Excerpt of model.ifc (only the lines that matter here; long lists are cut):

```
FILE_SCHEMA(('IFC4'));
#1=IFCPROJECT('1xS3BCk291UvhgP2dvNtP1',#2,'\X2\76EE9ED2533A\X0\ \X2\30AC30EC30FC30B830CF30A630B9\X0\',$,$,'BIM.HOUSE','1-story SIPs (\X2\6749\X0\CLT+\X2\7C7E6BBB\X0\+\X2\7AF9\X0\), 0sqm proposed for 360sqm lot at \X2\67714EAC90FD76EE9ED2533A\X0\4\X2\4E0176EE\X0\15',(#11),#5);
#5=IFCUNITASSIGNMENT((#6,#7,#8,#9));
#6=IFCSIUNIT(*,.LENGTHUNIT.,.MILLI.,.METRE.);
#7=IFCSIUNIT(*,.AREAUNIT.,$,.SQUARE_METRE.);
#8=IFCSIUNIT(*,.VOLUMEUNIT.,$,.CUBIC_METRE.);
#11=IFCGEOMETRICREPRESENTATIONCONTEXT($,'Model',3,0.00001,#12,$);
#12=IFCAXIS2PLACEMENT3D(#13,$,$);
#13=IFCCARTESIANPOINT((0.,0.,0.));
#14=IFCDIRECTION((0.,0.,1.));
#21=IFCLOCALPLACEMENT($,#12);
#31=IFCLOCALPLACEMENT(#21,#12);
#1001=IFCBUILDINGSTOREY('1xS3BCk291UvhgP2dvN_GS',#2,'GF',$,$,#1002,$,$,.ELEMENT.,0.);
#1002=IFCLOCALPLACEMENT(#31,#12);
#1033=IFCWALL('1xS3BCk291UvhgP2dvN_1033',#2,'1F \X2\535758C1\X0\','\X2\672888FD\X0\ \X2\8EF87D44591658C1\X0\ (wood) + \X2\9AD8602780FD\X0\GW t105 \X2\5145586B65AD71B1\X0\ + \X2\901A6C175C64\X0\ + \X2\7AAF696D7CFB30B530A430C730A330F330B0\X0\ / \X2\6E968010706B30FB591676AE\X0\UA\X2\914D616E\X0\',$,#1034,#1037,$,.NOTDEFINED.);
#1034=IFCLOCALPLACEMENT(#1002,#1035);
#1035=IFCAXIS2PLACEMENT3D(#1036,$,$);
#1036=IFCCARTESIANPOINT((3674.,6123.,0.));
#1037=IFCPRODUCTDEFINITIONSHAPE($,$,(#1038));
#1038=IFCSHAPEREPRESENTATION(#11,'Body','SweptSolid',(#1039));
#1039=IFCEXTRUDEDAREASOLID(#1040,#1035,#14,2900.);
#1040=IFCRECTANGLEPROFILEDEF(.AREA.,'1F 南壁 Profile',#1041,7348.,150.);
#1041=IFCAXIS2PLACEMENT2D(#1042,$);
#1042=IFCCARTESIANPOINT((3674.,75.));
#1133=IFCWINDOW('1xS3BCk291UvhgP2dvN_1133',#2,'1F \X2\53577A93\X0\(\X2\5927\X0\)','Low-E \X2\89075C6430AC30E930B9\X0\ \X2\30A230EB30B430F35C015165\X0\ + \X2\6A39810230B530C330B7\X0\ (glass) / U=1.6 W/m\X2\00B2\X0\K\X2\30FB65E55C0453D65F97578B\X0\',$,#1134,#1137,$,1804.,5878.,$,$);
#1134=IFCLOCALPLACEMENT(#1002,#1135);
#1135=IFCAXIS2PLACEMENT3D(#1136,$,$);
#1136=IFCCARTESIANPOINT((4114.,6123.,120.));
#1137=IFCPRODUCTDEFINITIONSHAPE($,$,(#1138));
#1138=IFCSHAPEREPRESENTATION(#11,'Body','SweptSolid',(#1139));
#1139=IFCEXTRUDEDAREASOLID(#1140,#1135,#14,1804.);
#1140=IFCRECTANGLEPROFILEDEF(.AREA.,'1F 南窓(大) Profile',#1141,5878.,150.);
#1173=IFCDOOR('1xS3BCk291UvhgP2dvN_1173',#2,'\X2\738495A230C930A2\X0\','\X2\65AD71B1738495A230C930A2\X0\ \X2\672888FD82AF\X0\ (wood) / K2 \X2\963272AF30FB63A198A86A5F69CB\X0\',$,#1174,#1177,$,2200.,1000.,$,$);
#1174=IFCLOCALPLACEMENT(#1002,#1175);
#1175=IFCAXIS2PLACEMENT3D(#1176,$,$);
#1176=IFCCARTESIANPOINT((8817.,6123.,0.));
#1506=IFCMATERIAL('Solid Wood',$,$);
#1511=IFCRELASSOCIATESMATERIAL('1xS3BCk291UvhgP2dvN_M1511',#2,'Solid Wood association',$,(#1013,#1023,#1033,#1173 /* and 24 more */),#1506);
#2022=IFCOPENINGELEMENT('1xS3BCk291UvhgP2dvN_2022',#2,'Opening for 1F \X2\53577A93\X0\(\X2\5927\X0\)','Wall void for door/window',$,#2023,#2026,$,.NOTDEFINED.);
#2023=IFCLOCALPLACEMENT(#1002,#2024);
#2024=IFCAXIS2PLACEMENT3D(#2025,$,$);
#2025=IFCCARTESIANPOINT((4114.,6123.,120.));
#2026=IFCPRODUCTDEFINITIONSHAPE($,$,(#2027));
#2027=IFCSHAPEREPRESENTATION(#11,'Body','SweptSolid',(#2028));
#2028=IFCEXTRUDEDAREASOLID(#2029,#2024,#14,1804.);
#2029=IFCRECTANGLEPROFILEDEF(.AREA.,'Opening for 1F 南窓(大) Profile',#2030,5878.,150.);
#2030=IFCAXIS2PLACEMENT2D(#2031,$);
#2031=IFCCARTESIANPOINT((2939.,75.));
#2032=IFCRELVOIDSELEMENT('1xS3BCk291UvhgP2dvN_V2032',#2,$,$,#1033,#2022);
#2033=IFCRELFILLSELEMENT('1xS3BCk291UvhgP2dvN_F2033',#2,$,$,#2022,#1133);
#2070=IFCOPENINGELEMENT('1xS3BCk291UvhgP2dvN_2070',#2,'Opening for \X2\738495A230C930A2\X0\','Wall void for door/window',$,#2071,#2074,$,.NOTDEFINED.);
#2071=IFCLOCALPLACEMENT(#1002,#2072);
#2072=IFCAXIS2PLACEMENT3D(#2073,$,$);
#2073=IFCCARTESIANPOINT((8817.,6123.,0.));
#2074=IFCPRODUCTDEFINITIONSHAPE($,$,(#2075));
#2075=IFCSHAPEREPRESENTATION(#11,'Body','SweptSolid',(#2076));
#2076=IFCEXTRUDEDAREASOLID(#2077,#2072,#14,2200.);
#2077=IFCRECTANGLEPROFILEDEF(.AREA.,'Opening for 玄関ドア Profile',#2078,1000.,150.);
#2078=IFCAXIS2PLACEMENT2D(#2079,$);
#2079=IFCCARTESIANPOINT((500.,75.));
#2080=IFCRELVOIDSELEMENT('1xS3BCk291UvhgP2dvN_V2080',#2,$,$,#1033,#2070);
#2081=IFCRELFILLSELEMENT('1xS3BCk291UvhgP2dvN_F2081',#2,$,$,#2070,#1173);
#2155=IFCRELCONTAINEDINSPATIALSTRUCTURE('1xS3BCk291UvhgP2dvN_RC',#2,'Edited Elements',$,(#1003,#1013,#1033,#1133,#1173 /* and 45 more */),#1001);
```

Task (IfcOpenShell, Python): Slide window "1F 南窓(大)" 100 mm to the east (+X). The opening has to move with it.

```python
import ifcopenshell
import ifcopenshell.api.geometry
import ifcopenshell.util.placement

model = ifcopenshell.open("model.ifc")

window = model.by_guid("1xS3BCk291UvhgP2dvN_1133")
opening = window.FillsVoids[0].RelatingOpeningElement
wall = opening.VoidsElements[0].RelatingBuildingElement

wall_matrix = ifcopenshell.util.placement.get_local_placement(wall.ObjectPlacement)
shift = wall_matrix[:3, 0] * 100.0
before = ifcopenshell.util.placement.get_local_placement(window.ObjectPlacement)[:3, 3].copy()

# The window is not placed relative to its opening, so move both.
for product in (opening, window):
    matrix = ifcopenshell.util.placement.get_local_placement(product.ObjectPlacement)
    matrix[:3, 3] += shift
    ifcopenshell.api.geometry.edit_object_placement(model, product=product, matrix=matrix, is_si=False)

after = ifcopenshell.util.placement.get_local_placement(window.ObjectPlacement)[:3, 3]
print("window moved by", (after - before).round(3) + 0.0)

model.write("model_updated.ifc")
```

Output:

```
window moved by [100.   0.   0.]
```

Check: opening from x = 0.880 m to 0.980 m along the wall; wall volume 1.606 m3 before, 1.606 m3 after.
